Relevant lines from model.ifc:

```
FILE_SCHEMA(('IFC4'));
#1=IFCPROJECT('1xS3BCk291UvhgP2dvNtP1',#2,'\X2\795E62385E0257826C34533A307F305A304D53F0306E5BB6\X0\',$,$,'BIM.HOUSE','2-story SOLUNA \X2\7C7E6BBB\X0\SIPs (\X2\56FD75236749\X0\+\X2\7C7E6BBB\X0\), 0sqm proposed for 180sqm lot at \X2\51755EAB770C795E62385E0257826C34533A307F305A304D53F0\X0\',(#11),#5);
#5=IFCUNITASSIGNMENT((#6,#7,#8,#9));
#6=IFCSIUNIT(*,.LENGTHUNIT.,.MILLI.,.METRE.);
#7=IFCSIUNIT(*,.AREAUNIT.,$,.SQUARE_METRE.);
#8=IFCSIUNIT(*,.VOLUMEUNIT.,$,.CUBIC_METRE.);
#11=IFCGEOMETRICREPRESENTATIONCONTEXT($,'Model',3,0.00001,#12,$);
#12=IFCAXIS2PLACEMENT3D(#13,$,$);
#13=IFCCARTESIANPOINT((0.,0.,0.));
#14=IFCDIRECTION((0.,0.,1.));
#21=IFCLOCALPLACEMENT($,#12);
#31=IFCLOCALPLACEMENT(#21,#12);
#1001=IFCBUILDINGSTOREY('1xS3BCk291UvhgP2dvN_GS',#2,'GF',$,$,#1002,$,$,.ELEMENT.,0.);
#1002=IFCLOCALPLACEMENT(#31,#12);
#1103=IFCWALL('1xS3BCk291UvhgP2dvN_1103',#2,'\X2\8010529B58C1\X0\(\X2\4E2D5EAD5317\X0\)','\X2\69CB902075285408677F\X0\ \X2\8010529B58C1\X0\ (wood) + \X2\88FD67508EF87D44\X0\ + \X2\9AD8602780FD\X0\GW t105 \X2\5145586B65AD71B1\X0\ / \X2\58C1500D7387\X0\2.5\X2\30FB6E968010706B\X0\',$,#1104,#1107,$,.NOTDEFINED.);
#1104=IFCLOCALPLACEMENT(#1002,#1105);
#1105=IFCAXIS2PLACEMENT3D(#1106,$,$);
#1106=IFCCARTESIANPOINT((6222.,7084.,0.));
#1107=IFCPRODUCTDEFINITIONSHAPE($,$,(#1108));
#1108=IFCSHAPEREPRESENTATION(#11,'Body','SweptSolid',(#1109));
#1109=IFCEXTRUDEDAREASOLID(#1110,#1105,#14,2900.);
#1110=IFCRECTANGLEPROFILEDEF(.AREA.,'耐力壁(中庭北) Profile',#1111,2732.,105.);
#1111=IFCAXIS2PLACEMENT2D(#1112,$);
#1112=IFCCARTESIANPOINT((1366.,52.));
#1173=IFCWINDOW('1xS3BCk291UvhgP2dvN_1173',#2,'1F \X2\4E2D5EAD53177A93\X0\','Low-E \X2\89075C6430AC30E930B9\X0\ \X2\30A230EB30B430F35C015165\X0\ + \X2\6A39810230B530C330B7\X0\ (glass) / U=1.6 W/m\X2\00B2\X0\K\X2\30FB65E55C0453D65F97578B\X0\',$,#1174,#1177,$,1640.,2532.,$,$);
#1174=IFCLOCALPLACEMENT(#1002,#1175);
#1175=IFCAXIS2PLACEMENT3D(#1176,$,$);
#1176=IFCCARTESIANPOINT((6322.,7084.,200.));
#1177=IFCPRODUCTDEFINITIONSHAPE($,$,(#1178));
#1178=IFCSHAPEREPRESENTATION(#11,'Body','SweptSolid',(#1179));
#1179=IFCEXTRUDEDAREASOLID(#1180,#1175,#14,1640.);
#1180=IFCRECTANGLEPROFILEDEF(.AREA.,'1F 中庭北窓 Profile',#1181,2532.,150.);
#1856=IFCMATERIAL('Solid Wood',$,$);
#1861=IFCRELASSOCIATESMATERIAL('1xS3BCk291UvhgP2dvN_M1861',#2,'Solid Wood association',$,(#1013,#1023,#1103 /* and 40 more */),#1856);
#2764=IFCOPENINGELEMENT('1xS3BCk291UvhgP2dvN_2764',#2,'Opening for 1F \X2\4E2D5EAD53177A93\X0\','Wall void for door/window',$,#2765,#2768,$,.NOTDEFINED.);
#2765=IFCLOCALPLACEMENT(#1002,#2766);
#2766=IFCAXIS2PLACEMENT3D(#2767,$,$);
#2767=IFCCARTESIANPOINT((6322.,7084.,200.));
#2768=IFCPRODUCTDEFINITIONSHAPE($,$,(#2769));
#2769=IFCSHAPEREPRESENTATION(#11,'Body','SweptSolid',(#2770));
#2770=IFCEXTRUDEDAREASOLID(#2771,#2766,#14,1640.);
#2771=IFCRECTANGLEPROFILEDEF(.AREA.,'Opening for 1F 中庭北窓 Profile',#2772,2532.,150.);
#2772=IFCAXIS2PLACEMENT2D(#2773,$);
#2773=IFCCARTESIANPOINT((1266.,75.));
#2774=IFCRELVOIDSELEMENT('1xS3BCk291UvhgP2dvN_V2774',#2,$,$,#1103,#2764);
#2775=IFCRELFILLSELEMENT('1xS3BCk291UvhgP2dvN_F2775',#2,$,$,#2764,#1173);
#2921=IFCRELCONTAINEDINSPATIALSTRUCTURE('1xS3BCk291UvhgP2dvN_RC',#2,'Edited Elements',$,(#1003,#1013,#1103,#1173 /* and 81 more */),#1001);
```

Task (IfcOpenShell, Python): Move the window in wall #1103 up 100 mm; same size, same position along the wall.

```python
import numpy as np
import ifcopenshell
import ifcopenshell.api.geometry
import ifcopenshell.util.placement
import ifcopenshell.util.unit

model = ifcopenshell.open("model.ifc")
unit_scale = ifcopenshell.util.unit.calculate_unit_scale(model)

window = model.by_guid("1xS3BCk291UvhgP2dvN_1173")
opening = window.FillsVoids[0].RelatingOpeningElement
dz = 100.0

shift = np.array([0.0, 0.0, dz])
# The window is not placed relative to its opening, so move both.
for product in (opening, window):
    matrix = ifcopenshell.util.placement.get_local_placement(product.ObjectPlacement)
    matrix[:3, 3] += shift
    ifcopenshell.api.geometry.edit_object_placement(model, product=product, matrix=matrix, is_si=False)

print(f"moved by {dz * unit_scale:+.3f} m")

model.write("model-out.ifc")
```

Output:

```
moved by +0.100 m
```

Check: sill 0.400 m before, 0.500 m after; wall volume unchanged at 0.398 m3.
